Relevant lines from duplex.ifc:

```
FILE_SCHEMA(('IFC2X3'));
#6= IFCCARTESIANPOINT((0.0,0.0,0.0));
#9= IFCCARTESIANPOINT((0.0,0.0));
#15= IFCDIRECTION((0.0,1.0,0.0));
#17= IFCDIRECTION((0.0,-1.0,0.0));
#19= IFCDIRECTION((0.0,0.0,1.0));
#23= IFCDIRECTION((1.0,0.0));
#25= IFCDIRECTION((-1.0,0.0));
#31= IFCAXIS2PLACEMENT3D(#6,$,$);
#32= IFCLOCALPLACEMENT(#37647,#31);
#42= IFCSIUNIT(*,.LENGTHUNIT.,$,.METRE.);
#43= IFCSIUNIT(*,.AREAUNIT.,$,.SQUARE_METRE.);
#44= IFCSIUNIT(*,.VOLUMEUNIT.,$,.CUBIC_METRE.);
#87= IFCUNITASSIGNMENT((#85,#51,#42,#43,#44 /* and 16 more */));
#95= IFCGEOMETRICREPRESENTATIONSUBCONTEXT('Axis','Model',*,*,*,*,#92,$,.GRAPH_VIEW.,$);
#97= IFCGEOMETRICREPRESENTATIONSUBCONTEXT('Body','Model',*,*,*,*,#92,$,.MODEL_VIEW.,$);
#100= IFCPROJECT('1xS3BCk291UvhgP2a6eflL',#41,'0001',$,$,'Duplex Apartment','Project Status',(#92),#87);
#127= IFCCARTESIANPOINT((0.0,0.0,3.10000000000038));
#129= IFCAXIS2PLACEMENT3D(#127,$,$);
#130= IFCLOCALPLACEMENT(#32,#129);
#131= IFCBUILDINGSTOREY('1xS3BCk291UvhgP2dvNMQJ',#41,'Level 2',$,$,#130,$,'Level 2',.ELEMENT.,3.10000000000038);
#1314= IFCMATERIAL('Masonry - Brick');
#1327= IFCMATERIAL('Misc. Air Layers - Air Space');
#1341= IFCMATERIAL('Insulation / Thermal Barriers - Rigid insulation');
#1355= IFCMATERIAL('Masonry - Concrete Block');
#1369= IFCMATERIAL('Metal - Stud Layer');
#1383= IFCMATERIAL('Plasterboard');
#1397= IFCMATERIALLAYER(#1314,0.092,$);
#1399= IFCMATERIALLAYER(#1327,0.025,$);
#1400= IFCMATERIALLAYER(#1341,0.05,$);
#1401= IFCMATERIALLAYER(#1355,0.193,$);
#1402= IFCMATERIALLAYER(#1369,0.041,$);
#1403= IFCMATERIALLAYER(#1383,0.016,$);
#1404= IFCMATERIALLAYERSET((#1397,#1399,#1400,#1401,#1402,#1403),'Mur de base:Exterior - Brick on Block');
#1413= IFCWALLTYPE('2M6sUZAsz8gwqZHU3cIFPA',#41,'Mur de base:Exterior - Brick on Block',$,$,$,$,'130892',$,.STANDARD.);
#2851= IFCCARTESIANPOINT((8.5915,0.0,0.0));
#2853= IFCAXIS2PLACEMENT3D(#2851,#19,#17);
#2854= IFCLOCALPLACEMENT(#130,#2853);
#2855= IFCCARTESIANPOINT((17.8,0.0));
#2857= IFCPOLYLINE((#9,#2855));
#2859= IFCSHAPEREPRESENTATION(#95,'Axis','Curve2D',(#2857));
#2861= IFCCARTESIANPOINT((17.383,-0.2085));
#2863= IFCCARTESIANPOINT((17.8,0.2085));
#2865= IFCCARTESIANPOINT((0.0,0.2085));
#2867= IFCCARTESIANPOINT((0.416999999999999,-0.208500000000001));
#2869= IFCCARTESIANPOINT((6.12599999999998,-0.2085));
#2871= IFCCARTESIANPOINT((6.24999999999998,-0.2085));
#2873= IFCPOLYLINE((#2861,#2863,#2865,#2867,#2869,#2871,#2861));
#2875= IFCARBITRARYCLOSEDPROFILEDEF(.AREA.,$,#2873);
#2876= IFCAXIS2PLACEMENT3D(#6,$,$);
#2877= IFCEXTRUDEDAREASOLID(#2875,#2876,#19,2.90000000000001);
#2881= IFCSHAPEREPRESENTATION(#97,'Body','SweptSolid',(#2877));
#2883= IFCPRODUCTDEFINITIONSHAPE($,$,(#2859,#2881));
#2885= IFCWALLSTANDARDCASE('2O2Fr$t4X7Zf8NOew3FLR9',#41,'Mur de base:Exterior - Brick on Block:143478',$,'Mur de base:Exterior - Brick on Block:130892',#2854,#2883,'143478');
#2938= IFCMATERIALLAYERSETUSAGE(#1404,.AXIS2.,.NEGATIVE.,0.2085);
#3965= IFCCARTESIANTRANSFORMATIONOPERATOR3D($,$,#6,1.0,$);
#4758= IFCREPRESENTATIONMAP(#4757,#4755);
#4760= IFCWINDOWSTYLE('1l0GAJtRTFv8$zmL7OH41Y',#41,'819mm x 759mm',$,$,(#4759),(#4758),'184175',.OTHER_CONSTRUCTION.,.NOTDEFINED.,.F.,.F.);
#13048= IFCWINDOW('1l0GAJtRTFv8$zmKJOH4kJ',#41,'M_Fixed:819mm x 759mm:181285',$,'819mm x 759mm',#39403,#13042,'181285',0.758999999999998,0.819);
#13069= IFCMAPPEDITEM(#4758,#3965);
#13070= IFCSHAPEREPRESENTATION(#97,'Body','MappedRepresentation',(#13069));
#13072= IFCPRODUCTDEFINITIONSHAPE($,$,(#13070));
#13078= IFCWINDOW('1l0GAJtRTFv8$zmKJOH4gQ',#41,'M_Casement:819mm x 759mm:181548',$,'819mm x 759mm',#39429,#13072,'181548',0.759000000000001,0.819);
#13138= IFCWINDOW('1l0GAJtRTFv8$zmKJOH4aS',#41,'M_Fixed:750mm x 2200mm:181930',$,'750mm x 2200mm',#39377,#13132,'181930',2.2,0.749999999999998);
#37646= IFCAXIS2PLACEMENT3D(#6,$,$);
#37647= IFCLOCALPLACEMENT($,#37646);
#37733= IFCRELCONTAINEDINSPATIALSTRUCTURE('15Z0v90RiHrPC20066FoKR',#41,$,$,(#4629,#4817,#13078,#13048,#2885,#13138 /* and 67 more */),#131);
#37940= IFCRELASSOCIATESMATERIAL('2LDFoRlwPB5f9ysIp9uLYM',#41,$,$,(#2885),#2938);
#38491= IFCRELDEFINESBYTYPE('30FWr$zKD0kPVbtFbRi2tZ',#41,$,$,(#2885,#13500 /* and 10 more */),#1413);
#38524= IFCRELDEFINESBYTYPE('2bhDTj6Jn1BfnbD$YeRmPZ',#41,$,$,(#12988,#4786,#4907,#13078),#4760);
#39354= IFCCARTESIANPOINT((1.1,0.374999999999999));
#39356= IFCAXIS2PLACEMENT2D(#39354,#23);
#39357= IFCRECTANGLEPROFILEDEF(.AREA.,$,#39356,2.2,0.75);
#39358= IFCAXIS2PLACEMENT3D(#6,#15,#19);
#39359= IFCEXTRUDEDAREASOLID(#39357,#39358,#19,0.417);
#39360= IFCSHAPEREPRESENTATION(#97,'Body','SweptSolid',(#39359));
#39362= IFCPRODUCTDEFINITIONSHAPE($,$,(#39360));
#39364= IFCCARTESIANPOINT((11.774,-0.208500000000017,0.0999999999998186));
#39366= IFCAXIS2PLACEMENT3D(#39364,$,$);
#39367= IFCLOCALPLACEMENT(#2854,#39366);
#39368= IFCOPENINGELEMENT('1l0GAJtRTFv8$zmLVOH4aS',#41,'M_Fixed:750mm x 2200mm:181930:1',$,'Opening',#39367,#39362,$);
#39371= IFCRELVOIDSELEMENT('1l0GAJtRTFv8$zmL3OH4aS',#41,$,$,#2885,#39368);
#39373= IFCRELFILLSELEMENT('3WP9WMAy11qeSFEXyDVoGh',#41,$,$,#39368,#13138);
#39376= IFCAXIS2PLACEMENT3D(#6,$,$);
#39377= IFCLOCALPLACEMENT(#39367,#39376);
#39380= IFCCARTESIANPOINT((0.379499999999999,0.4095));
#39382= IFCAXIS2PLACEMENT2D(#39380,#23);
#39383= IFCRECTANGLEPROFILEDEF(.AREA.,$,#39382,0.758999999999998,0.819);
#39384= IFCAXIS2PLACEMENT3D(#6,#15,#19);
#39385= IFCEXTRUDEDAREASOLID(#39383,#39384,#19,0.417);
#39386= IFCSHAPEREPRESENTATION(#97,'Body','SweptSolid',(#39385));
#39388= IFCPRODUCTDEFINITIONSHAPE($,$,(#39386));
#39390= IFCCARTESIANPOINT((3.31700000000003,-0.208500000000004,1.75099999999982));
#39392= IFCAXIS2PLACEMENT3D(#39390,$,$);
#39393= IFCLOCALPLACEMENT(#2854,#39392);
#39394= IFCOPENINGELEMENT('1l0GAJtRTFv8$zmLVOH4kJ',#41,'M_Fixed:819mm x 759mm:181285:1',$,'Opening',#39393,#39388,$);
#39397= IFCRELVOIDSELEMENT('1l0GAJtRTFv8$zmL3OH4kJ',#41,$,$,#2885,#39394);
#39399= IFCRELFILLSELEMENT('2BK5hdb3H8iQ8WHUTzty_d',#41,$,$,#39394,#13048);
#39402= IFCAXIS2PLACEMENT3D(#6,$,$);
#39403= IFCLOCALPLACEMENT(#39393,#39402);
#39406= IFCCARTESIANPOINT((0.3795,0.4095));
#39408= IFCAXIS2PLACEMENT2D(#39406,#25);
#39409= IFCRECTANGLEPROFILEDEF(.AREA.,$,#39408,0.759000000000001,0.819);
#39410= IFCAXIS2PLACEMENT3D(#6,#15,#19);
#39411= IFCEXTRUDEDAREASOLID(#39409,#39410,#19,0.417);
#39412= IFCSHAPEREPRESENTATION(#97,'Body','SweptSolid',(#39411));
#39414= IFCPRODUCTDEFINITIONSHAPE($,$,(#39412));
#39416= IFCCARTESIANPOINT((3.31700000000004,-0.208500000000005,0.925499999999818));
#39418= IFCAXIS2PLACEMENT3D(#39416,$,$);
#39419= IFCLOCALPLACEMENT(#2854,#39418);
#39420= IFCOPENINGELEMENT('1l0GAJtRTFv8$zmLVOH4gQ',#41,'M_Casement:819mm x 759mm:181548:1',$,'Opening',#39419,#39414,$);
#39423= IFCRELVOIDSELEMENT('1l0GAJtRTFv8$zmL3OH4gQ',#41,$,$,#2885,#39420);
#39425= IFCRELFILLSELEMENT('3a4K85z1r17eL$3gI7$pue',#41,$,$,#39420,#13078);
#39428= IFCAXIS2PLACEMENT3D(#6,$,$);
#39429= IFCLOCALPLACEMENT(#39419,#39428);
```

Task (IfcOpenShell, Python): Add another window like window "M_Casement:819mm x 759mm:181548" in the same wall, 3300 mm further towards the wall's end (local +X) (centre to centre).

```python
import ifcopenshell
import ifcopenshell.api.feature
import ifcopenshell.api.geometry
import ifcopenshell.api.root
import ifcopenshell.geom
import ifcopenshell.util.element
import ifcopenshell.util.placement
import ifcopenshell.util.shape
import ifcopenshell.util.unit

model = ifcopenshell.open("duplex.ifc")
unit_scale = ifcopenshell.util.unit.calculate_unit_scale(model)
settings = ifcopenshell.geom.settings()


def volume(element):
    """Net volume in cubic metres, openings subtracted."""
    shape = ifcopenshell.geom.create_shape(settings, element)
    return ifcopenshell.util.shape.get_volume(shape.geometry)


def reuse_history(source, copy):
    """copy_class also copies each property set's owner history, people and application; keep the originals."""
    for rel in copy.IsDefinedBy:
        if rel.is_a("IfcRelDefinesByProperties") and (history := rel.RelatingPropertyDefinition.OwnerHistory):
            rel.RelatingPropertyDefinition.OwnerHistory = source.OwnerHistory
            ifcopenshell.util.element.remove_deep2(model, history)


window = model.by_id(13078)
opening = window.FillsVoids[0].RelatingOpeningElement
wall = opening.VoidsElements[0].RelatingBuildingElement
before = volume(wall)
shift = ifcopenshell.util.placement.get_local_placement(wall.ObjectPlacement)[:3, 0] * 3.3 / unit_scale

# copy_class copies the void relationship, type, container and properties, but no geometry.
new_opening = ifcopenshell.api.root.copy_class(model, product=opening)
new_opening.Representation = ifcopenshell.util.element.copy_deep(
    model, opening.Representation, exclude=["IfcGeometricRepresentationContext", "IfcRepresentationMap"]
)
new_opening.Name = "M_Casement:819mm x 759mm"
new_window = ifcopenshell.api.root.copy_class(model, product=window)
new_window.Representation = ifcopenshell.util.element.copy_deep(
    model, window.Representation, exclude=["IfcGeometricRepresentationContext", "IfcRepresentationMap"]
)
new_window.Name = "M_Casement:819mm x 759mm"
new_window.Tag = None
reuse_history(window, new_window)
fills = ifcopenshell.api.feature.add_filling(model, opening=new_opening, element=new_window)
fills.OwnerHistory = new_window.OwnerHistory  # required in IFC2X3

for old, new in ((opening, new_opening), (window, new_window)):
    matrix = ifcopenshell.util.placement.get_local_placement(old.ObjectPlacement)
    matrix[:3, 3] += shift
    ifcopenshell.api.geometry.edit_object_placement(model, product=new, matrix=matrix, is_si=False)

after = volume(wall)

print(f"wall volume {before:.3f} -> {after:.3f} m3")

model.write("duplex_updated.ifc")
```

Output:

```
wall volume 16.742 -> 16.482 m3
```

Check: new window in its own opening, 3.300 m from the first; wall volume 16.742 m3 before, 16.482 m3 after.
